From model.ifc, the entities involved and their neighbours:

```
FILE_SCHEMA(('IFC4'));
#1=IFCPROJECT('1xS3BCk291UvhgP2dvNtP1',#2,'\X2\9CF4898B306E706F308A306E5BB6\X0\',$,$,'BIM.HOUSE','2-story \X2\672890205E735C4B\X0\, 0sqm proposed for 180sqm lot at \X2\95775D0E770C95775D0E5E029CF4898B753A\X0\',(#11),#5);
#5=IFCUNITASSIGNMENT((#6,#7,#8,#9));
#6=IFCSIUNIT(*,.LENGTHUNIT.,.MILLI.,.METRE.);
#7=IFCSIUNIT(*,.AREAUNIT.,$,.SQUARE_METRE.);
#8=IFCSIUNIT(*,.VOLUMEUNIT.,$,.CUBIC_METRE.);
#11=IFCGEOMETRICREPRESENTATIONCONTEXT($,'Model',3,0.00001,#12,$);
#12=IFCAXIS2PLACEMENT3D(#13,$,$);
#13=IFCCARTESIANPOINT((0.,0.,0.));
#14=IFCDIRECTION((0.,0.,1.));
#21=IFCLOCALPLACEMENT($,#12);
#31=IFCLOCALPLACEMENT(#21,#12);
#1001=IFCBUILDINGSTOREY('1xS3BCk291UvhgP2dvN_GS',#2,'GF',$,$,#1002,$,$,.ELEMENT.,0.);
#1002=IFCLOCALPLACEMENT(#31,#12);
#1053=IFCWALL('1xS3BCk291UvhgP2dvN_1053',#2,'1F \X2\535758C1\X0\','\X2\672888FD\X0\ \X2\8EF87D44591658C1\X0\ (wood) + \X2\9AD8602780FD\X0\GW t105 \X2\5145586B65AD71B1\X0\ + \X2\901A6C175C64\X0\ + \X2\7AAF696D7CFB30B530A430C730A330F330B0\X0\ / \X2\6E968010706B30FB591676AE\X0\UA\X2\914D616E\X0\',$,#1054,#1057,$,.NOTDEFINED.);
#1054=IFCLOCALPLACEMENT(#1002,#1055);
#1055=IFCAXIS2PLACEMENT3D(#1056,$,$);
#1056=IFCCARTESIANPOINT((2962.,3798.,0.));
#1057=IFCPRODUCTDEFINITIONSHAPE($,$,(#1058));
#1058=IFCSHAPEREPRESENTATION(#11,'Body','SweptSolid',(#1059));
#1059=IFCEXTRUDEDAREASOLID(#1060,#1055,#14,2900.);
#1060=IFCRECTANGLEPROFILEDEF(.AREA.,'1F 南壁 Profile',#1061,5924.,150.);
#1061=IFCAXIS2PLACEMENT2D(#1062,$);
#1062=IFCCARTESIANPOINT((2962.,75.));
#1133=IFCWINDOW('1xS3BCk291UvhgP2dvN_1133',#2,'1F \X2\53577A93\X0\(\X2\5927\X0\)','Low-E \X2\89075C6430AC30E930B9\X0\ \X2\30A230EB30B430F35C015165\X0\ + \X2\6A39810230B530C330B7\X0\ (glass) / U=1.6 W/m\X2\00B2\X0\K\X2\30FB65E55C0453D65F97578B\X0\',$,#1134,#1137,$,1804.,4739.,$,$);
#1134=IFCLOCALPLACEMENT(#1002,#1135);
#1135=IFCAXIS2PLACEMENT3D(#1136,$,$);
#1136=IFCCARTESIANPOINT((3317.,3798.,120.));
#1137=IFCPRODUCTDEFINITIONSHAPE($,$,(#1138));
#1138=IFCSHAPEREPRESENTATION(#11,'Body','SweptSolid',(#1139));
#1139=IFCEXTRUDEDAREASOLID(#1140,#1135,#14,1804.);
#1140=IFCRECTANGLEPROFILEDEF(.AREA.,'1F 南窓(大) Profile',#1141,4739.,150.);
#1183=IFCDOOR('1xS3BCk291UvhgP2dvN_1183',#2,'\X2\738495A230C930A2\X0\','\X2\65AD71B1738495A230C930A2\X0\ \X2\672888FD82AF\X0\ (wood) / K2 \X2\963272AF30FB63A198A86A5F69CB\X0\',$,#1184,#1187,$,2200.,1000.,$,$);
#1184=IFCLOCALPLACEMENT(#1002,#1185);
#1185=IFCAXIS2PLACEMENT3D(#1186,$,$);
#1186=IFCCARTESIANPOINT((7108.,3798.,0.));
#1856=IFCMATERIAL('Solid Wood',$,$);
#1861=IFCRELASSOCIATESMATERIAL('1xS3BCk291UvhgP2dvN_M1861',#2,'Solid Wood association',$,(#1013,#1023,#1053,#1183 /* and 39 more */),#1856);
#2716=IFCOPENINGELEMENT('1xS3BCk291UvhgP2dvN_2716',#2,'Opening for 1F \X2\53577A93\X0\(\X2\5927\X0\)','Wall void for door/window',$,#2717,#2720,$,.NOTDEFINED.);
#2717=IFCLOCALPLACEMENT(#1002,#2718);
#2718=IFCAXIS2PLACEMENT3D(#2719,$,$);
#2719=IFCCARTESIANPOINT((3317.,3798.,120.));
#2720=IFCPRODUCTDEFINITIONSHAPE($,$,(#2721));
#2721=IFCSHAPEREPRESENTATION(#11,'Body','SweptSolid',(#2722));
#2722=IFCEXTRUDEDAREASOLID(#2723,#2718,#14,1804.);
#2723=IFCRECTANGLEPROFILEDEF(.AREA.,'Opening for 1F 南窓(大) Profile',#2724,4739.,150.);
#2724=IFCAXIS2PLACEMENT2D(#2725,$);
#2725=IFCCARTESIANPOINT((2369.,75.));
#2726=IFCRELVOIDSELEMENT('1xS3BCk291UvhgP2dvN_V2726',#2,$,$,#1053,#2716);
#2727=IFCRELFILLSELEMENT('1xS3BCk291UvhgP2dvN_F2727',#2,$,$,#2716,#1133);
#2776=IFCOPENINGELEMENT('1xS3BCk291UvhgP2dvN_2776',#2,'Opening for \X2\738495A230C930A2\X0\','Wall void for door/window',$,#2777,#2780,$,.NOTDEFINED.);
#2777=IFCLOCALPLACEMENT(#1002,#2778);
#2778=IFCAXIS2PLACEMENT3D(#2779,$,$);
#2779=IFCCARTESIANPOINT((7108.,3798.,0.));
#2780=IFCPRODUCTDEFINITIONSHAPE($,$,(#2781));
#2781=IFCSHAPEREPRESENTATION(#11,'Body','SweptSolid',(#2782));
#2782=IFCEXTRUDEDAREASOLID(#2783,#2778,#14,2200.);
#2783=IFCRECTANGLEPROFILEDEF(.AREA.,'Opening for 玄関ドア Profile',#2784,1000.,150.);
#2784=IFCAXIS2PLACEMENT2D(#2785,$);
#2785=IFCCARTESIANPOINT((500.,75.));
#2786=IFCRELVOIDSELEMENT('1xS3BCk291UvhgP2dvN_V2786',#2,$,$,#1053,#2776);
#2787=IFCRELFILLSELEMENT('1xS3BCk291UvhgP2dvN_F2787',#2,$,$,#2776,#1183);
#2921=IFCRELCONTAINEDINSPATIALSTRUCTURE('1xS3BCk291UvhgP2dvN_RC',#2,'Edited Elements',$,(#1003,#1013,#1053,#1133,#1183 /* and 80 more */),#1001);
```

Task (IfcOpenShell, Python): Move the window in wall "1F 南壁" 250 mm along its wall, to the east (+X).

```python
import ifcopenshell
import ifcopenshell.api.geometry
import ifcopenshell.util.placement

model = ifcopenshell.open("model.ifc")

window = model.by_guid("1xS3BCk291UvhgP2dvN_1133")
opening = window.FillsVoids[0].RelatingOpeningElement
wall = opening.VoidsElements[0].RelatingBuildingElement

wall_matrix = ifcopenshell.util.placement.get_local_placement(wall.ObjectPlacement)
shift = wall_matrix[:3, 0] * 250.0
before = ifcopenshell.util.placement.get_local_placement(window.ObjectPlacement)[:3, 3].copy()

# The window is not placed relative to its opening, so move both.
for product in (opening, window):
    matrix = ifcopenshell.util.placement.get_local_placement(product.ObjectPlacement)
    matrix[:3, 3] += shift
    ifcopenshell.api.geometry.edit_object_placement(model, product=product, matrix=matrix, is_si=False)

after = ifcopenshell.util.placement.get_local_placement(window.ObjectPlacement)[:3, 3]
print("window moved by", (after - before).round(3) + 0.0)

model.write("model_v2.ifc")
```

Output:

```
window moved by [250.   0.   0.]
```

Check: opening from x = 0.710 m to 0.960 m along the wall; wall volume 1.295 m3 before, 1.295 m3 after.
